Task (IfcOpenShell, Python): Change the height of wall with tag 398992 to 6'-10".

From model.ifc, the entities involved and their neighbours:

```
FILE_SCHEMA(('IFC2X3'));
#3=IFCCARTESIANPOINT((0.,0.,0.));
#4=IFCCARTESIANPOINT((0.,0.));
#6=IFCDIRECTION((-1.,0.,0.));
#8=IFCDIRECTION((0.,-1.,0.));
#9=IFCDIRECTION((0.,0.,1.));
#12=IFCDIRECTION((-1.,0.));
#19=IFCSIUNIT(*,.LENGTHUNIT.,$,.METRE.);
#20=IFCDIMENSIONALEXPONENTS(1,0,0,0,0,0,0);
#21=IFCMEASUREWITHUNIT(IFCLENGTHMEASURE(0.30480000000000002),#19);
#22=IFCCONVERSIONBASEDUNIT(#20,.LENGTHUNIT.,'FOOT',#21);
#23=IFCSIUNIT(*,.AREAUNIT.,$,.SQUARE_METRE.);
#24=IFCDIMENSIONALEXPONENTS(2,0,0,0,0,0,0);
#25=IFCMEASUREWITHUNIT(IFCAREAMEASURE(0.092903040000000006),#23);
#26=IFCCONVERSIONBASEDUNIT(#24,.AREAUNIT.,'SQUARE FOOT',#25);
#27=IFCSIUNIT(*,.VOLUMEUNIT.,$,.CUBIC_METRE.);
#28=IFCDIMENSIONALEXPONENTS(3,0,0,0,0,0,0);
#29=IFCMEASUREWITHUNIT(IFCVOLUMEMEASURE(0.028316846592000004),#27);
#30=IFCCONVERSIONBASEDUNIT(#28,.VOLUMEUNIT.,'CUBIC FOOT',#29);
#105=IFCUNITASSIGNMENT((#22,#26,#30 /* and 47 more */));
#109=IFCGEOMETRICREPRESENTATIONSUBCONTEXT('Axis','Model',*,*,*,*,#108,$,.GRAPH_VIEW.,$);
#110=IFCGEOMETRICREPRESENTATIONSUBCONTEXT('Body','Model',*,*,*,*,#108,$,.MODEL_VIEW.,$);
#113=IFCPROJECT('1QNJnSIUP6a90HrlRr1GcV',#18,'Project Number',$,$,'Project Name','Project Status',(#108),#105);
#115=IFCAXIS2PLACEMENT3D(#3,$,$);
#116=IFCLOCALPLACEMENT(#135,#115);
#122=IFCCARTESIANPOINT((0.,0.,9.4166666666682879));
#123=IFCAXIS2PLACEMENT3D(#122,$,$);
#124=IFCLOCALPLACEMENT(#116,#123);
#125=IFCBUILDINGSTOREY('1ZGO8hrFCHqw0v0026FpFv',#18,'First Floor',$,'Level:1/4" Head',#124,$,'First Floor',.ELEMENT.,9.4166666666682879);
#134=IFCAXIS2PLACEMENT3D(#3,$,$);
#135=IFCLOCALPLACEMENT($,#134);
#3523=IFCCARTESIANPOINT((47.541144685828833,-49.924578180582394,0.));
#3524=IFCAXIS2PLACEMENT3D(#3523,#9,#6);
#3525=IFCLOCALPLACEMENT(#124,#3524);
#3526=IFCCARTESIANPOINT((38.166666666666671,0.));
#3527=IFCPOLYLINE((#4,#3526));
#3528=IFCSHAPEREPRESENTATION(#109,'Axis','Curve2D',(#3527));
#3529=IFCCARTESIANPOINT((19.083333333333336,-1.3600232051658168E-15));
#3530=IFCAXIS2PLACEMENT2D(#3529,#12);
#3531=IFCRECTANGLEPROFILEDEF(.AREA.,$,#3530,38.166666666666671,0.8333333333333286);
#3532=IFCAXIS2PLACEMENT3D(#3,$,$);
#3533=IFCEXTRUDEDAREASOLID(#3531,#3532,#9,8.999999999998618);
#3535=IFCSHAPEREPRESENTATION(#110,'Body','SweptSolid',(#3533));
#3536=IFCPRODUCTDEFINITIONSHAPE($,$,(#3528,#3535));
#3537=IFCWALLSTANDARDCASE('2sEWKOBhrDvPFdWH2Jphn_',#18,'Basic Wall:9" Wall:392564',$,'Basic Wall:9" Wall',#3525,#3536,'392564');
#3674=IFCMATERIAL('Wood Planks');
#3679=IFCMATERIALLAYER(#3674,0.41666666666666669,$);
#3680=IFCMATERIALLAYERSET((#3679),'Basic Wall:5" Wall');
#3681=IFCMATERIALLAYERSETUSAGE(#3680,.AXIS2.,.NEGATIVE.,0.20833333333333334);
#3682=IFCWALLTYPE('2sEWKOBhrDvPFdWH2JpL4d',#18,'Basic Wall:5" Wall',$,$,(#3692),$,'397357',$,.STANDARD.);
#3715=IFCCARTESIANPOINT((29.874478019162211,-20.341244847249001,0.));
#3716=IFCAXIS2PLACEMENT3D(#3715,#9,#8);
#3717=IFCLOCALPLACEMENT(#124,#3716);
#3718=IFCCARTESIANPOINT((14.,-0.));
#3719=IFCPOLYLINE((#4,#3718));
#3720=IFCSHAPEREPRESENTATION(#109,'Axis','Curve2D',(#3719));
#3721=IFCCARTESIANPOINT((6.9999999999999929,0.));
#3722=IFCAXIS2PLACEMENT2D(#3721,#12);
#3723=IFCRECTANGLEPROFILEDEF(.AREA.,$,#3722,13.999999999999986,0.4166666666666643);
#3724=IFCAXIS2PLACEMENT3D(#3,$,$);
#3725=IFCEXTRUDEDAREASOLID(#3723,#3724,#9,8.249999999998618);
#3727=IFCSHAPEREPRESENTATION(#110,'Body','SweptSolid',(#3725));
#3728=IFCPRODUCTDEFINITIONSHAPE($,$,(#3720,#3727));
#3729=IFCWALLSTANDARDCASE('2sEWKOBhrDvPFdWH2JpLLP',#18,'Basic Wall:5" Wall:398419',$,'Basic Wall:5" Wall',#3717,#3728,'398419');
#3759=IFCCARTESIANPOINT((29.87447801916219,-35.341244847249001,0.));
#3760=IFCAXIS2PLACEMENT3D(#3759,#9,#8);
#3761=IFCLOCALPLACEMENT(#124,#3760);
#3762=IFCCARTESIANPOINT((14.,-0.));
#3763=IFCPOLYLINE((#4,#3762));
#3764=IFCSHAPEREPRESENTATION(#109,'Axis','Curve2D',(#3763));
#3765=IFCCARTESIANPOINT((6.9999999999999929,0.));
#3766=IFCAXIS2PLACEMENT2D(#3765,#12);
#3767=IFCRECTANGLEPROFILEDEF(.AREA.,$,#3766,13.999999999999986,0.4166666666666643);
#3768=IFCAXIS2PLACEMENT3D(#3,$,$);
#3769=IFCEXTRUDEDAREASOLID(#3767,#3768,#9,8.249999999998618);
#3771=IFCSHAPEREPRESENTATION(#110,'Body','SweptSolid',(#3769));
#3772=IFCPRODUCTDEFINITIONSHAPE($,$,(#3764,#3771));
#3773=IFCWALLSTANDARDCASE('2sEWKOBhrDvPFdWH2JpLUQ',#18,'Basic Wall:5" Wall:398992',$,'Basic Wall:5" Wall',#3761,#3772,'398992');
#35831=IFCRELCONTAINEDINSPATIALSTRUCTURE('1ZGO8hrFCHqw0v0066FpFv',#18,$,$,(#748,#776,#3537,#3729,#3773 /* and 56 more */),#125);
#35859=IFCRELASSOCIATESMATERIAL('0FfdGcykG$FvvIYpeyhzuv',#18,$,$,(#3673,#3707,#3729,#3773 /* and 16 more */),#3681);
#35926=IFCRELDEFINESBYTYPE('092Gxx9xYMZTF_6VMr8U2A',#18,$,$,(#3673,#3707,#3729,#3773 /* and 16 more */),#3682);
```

```python
import ifcopenshell
import ifcopenshell.geom
import ifcopenshell.util.representation
import ifcopenshell.util.shape
import ifcopenshell.util.unit

model = ifcopenshell.open("model.ifc")
unit_scale = ifcopenshell.util.unit.calculate_unit_scale(model)
settings = ifcopenshell.geom.settings()


def volume(element):
    """Net volume in cubic metres, openings subtracted."""
    shape = ifcopenshell.geom.create_shape(settings, element)
    return ifcopenshell.util.shape.get_volume(shape.geometry)


wall = model.by_guid("2sEWKOBhrDvPFdWH2JpLUQ")
before = volume(wall)

body = ifcopenshell.util.representation.get_representation(wall, "Model", "Body")
solid = body.Items[0]
old_height = solid.Depth
solid.Depth = 82 * 0.0254 / unit_scale
after = volume(wall)

print(f"height {old_height:g} -> {solid.Depth:g}, volume {before:.3f} -> {after:.3f} m3")

model.write("model_edited.ifc")
```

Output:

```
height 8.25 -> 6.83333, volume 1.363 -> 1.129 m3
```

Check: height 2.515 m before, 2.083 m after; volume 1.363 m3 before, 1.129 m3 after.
